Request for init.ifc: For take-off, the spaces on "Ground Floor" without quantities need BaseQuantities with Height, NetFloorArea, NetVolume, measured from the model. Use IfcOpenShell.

First a look at what the model holds.

```python
import ifcopenshell
import ifcopenshell.util.element
import ifcopenshell.util.unit

model = ifcopenshell.open("init.ifc")
print(model.schema)
for unit_type in ("LENGTHUNIT", "AREAUNIT", "VOLUMEUNIT"):
    print(unit_type, ifcopenshell.util.unit.calculate_unit_scale(model, unit_type))
storey = next(s for s in model.by_type("IfcBuildingStorey") if s.Name == "Ground Floor")
spaces = [e for e in ifcopenshell.util.element.get_decomposition(storey) if e.is_a("IfcSpace")]
for e in sorted(spaces, key=lambda e: e.id()):
    print(e.id(), e.is_a(), e.Name, list(ifcopenshell.util.element.get_psets(e, qtos_only=True)), sep=" | ")
```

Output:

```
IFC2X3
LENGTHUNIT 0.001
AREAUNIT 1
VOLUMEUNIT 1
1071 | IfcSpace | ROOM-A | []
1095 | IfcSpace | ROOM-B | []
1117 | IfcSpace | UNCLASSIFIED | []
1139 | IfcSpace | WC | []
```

```python
import ifcopenshell
import ifcopenshell.api.pset
import ifcopenshell.geom
import ifcopenshell.util.element
import ifcopenshell.util.shape
import ifcopenshell.util.unit

model = ifcopenshell.open("init.ifc")
unit_scale = ifcopenshell.util.unit.calculate_unit_scale(model)
area_scale = ifcopenshell.util.unit.calculate_unit_scale(model, "AREAUNIT")
volume_scale = ifcopenshell.util.unit.calculate_unit_scale(model, "VOLUMEUNIT")
settings = ifcopenshell.geom.settings()

storey = next(s for s in model.by_type("IfcBuildingStorey") if s.Name == "Ground Floor")
spaces = [e for e in ifcopenshell.util.element.get_decomposition(storey) if e.is_a("IfcSpace")]

for e in sorted(spaces, key=lambda e: e.id()):
    if ifcopenshell.util.element.get_psets(e, qtos_only=True, should_inherit=False):
        continue
    # Geometry comes back in metres, in the element's own axes.
    shape = ifcopenshell.geom.create_shape(settings, e)
    values = {
        "Height": ifcopenshell.util.shape.get_z(shape.geometry) / unit_scale,
        "NetFloorArea": ifcopenshell.util.shape.get_footprint_area(shape.geometry) / area_scale,
        "NetVolume": ifcopenshell.util.shape.get_volume(shape.geometry) / volume_scale,
    }
    qto = ifcopenshell.api.pset.add_qto(model, product=e, name="BaseQuantities")
    ifcopenshell.api.pset.edit_qto(model, qto=qto, properties=values)
    print(e.id(), {k: round(v, 3) for k, v in values.items()})

model.write("init_rev.ifc")
```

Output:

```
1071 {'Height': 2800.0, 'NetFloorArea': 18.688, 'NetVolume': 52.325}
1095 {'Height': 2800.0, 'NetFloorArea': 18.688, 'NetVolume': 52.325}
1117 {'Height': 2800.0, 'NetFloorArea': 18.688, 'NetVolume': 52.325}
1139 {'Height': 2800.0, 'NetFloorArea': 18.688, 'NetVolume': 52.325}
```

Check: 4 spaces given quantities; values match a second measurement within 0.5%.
